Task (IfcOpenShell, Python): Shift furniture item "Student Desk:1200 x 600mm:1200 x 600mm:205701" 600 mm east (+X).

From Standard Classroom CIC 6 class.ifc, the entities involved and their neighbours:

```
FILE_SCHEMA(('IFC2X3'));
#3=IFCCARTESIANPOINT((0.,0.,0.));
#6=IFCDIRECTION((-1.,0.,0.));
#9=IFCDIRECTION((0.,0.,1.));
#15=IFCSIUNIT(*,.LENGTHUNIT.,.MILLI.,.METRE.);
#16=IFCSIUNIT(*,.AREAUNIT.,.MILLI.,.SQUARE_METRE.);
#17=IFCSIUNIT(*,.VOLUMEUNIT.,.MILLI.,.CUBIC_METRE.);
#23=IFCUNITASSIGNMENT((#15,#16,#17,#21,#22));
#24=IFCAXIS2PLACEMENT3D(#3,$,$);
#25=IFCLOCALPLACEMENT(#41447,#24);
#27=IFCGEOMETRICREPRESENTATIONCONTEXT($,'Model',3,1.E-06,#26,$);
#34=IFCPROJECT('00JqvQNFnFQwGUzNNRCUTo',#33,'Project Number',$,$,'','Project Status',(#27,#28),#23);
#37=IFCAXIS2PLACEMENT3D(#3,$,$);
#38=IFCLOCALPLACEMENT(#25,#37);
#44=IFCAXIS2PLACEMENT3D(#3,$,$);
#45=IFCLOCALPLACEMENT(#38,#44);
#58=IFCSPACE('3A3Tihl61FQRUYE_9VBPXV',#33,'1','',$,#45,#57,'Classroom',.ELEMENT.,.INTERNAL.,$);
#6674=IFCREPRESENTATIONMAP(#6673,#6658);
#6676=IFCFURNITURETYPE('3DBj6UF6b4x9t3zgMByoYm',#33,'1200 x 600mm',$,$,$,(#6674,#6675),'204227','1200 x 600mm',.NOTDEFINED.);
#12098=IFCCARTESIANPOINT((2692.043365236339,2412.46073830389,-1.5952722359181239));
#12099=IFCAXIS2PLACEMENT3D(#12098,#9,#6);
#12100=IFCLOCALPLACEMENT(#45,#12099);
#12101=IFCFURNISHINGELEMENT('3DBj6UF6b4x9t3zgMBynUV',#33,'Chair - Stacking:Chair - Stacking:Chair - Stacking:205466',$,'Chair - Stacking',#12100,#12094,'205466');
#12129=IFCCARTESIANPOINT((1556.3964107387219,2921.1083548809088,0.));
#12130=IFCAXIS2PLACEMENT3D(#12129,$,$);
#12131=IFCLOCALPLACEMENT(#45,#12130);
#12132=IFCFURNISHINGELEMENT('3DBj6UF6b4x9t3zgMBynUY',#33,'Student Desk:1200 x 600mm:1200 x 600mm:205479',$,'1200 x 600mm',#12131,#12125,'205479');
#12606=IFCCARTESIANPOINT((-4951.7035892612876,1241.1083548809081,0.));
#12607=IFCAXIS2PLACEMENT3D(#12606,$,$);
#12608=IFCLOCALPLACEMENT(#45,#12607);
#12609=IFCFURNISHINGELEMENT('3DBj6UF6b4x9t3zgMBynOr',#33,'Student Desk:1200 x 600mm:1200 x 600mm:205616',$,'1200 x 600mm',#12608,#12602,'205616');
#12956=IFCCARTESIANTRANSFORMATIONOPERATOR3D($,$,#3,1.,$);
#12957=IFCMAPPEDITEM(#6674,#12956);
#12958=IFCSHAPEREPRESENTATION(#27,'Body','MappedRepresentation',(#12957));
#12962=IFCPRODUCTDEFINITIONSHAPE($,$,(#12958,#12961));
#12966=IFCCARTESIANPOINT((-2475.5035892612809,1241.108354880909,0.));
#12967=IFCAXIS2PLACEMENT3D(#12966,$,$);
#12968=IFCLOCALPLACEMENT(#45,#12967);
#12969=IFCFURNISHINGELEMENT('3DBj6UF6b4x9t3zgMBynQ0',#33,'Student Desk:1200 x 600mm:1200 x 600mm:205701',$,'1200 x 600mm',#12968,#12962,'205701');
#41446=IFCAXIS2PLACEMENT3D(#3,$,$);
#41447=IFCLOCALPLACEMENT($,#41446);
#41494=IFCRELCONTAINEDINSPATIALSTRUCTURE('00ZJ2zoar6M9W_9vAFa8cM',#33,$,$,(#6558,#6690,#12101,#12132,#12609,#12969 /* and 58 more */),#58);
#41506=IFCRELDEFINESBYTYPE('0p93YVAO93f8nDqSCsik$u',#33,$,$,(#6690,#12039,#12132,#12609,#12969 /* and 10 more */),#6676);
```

```python
import ifcopenshell
import ifcopenshell.api.geometry
import ifcopenshell.util.placement

model = ifcopenshell.open("Standard Classroom CIC 6 class.ifc")

item = model.by_guid("3DBj6UF6b4x9t3zgMBynQ0")
matrix = ifcopenshell.util.placement.get_local_placement(item.ObjectPlacement)
matrix[0, 3] += 600.0
ifcopenshell.api.geometry.edit_object_placement(model, product=item, matrix=matrix, is_si=False)

print(ifcopenshell.util.placement.get_local_placement(item.ObjectPlacement).round(3) + 0.0)

model.write("Standard Classroom CIC 6 class_rev.ifc")
```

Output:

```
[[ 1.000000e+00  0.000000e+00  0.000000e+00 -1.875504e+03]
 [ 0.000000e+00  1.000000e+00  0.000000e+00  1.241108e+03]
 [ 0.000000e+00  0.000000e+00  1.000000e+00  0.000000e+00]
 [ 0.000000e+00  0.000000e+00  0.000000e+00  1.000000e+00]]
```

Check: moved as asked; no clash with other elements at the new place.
